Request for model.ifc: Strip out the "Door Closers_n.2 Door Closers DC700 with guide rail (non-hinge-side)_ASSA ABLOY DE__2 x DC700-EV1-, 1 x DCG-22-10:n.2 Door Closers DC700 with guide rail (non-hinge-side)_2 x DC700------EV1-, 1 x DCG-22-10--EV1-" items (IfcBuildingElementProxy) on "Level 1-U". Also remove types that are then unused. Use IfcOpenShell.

First a look at what the model holds.

```python
import ifcopenshell
import ifcopenshell.util.element

model = ifcopenshell.open("model.ifc")
print(model.schema)
storey = next(s for s in model.by_type("IfcBuildingStorey") if s.Name == "Level 1-U")
proxies = [e for e in ifcopenshell.util.element.get_decomposition(storey) if e.is_a("IfcBuildingElementProxy")]
seen = {}
for e in proxies:
    element_type = ifcopenshell.util.element.get_type(e)
    name = element_type.Name if element_type not in (None, e) else None
    seen[name] = seen.get(name, 0) + 1
for name, count in sorted(seen.items(), key=str):
    print(count, "x", name)
```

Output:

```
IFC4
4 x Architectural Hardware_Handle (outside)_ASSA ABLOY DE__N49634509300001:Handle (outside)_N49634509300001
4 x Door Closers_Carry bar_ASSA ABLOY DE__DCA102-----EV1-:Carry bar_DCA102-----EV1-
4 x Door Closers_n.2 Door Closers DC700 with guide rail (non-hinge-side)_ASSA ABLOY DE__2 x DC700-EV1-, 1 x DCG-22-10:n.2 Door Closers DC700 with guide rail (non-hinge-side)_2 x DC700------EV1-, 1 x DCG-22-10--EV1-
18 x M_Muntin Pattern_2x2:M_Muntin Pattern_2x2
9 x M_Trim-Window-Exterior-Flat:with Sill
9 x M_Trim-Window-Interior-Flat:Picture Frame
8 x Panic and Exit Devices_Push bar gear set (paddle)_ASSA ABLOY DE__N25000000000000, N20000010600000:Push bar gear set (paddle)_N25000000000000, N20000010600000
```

```python
import ifcopenshell
import ifcopenshell.api.root
import ifcopenshell.util.element

model = ifcopenshell.open("model.ifc")

storey = next(s for s in model.by_type("IfcBuildingStorey") if s.Name == "Level 1-U")
proxies = [e for e in ifcopenshell.util.element.get_decomposition(storey) if e.is_a("IfcBuildingElementProxy")]
targets = [e for e in proxies if (t := ifcopenshell.util.element.get_type(e)) not in (None, e) and t.Name == "Door Closers_n.2 Door Closers DC700 with guide rail (non-hinge-side)_ASSA ABLOY DE__2 x DC700-EV1-, 1 x DCG-22-10:n.2 Door Closers DC700 with guide rail (non-hinge-side)_2 x DC700------EV1-, 1 x DCG-22-10--EV1-"]
types = {ifcopenshell.util.element.get_type(e) for e in targets} - {None, *targets}

for e in targets:
    ifcopenshell.api.root.remove_product(model, product=e)
print(len(targets), "removed")

unused = [t for t in types if not ifcopenshell.util.element.get_types(t)]
for t in unused:
    ifcopenshell.api.root.remove_product(model, product=t)
print(len(unused), "unused types removed")

model.write("model_v2.ifc")
```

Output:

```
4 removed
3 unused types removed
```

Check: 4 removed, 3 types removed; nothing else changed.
